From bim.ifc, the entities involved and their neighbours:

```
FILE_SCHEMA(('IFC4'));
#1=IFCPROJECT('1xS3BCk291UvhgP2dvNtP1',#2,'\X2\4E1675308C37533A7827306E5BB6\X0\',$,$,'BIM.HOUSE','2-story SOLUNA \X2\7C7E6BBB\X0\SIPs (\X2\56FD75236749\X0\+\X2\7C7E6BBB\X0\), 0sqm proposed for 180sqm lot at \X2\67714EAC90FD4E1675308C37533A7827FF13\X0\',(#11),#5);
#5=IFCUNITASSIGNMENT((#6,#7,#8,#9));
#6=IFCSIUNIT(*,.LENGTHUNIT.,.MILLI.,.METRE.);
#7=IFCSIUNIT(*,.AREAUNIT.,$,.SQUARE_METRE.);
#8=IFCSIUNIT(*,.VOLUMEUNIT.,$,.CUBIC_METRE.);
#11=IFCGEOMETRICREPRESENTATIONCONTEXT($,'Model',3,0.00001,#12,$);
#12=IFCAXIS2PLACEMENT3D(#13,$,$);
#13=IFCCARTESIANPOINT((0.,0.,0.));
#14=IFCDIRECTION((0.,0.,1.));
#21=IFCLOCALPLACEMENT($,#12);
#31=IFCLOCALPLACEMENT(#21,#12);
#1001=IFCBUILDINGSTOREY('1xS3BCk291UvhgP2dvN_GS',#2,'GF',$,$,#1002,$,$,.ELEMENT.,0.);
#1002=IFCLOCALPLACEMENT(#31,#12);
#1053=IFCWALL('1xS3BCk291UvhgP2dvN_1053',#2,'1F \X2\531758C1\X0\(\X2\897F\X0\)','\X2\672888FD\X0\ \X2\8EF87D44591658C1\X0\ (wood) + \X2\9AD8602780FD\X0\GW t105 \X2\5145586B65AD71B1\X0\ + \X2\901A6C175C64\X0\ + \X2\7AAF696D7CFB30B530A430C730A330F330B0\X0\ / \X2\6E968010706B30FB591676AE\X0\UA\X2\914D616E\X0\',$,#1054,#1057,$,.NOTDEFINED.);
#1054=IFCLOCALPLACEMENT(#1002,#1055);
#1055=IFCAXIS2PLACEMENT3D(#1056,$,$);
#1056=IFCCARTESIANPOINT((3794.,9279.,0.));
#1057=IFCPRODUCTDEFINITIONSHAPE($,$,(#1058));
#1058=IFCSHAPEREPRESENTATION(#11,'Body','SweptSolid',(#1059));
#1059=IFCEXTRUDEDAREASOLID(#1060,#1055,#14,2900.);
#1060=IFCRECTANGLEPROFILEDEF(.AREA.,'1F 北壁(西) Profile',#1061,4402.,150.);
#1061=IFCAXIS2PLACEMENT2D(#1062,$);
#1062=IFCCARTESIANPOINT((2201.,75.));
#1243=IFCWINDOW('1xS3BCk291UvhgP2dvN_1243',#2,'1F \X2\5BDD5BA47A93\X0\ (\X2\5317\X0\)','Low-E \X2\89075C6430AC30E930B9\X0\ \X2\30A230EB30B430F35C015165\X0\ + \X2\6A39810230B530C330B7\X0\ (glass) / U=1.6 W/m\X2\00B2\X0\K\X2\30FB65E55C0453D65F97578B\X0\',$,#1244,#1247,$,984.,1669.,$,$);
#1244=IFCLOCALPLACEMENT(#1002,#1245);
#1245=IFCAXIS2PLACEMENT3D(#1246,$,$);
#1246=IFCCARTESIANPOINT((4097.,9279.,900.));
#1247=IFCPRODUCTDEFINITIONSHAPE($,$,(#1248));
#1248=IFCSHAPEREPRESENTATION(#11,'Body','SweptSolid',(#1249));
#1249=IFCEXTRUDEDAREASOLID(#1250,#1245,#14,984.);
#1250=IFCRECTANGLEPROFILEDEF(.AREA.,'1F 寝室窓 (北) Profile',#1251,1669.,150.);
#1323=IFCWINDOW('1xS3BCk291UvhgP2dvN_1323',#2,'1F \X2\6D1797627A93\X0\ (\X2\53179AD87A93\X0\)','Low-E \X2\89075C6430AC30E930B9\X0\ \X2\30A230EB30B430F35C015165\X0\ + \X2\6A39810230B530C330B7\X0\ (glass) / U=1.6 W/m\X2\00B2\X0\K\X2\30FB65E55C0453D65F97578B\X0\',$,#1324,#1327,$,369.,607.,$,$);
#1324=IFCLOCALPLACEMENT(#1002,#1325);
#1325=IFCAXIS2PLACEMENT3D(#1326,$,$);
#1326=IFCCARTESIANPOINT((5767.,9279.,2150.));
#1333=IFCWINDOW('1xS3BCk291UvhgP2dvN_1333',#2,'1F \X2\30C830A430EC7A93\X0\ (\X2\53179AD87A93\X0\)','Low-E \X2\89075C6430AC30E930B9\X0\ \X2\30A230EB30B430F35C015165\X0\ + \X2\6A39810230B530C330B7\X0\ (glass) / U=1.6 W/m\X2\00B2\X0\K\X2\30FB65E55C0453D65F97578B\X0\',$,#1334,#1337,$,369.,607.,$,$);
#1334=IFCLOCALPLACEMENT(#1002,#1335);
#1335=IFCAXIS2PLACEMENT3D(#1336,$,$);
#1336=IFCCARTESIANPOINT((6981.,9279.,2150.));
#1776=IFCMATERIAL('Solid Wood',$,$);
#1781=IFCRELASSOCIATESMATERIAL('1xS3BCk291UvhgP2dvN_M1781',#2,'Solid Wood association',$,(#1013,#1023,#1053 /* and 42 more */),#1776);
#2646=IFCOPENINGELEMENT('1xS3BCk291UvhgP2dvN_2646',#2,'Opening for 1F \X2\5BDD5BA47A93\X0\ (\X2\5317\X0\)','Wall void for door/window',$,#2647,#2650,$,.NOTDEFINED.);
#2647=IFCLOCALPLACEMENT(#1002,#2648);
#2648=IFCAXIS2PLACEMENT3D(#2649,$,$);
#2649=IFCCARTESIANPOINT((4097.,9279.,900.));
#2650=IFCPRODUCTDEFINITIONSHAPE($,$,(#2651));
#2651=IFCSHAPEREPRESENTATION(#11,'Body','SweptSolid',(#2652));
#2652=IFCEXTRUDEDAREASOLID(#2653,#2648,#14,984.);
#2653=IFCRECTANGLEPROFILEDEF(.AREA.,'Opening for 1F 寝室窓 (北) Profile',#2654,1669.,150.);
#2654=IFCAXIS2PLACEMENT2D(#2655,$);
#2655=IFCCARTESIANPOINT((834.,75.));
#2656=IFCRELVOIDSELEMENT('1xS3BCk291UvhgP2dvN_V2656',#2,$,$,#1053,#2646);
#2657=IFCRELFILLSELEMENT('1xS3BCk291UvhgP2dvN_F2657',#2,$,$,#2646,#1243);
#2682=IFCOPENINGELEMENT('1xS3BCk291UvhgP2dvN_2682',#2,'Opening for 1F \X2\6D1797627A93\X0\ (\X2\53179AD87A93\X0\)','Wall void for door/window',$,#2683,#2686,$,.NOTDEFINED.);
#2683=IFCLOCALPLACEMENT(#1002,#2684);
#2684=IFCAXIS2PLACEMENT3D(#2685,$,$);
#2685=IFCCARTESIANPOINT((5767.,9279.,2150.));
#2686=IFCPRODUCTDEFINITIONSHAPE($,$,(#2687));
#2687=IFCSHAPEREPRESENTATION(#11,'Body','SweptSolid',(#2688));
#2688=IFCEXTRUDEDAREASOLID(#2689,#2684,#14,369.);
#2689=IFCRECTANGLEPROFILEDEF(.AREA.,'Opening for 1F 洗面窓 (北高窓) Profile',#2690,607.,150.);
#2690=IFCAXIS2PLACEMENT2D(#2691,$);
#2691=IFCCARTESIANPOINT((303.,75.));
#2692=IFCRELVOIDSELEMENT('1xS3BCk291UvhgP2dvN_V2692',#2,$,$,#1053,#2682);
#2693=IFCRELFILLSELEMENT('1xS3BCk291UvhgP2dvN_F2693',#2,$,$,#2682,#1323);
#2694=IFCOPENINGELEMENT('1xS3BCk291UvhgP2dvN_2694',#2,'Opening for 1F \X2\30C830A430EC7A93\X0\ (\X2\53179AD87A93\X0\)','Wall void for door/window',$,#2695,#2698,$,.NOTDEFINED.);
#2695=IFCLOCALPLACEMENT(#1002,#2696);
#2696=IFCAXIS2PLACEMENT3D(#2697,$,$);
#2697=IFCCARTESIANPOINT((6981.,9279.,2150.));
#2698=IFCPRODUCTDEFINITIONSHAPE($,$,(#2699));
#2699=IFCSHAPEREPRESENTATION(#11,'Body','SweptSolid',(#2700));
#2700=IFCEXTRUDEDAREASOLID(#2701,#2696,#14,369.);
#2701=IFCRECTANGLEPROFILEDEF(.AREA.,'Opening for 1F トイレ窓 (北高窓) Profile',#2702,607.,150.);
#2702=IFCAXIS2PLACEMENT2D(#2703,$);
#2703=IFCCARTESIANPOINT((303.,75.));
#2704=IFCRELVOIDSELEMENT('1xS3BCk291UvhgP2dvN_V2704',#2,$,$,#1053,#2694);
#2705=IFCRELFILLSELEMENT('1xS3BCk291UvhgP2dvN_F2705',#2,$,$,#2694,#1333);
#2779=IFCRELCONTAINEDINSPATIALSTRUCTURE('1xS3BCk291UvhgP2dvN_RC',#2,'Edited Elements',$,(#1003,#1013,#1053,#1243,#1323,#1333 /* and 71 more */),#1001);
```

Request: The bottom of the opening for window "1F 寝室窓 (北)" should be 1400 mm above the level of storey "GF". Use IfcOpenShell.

```python
import numpy as np
import ifcopenshell
import ifcopenshell.api.geometry
import ifcopenshell.geom
import ifcopenshell.util.element
import ifcopenshell.util.placement
import ifcopenshell.util.shape
import ifcopenshell.util.unit

model = ifcopenshell.open("bim.ifc")
unit_scale = ifcopenshell.util.unit.calculate_unit_scale(model)

window = model.by_id(1243)
opening = window.FillsVoids[0].RelatingOpeningElement
storey = ifcopenshell.util.element.get_container(window, ifc_class="IfcBuildingStorey")
level = ifcopenshell.util.placement.get_local_placement(storey.ObjectPlacement)[2, 3]

# The opening's origin need not be at the sill, so measure its lowest point.
shape = ifcopenshell.geom.create_shape(ifcopenshell.geom.settings(), opening)
bottom = ifcopenshell.util.shape.get_shape_bottom_elevation(shape, shape.geometry) / unit_scale
dz = level + 1400.0 - bottom

shift = np.array([0.0, 0.0, dz])
# The window is not placed relative to its opening, so move both.
for product in (opening, window):
    matrix = ifcopenshell.util.placement.get_local_placement(product.ObjectPlacement)
    matrix[:3, 3] += shift
    ifcopenshell.api.geometry.edit_object_placement(model, product=product, matrix=matrix, is_si=False)

print(f"moved by {dz * unit_scale:+.3f} m")

model.write("bim-out.ifc")
```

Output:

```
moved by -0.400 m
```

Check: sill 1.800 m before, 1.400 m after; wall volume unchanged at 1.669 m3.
